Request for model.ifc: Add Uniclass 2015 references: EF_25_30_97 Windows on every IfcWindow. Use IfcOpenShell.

First a look at what the model holds.

```python
import ifcopenshell

model = ifcopenshell.open("model.ifc")
print(model.schema)
print("classifications:", [c.Name for c in model.by_type("IfcClassification")])
for ifc_class in ("IfcDoor", "IfcRoof", "IfcStair", "IfcWall", "IfcWindow"):
    print(ifc_class, len(model.by_type(ifc_class)))
```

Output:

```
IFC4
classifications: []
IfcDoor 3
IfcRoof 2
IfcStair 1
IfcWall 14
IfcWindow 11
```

```python
import ifcopenshell
import ifcopenshell.api.classification

model = ifcopenshell.open("model.ifc")

system = ifcopenshell.api.classification.add_classification(model, classification="Uniclass 2015")

codes = {
    "IfcWindow": ("EF_25_30_97", "Windows"),
}
for ifc_class, (code, name) in codes.items():
    products = model.by_type(ifc_class)
    ifcopenshell.api.classification.add_reference(
        model, products=products, classification=system, identification=code, name=name
    )
    print(code, len(products))

model.write("model_rev.ifc")
```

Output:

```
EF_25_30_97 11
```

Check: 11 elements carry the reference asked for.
